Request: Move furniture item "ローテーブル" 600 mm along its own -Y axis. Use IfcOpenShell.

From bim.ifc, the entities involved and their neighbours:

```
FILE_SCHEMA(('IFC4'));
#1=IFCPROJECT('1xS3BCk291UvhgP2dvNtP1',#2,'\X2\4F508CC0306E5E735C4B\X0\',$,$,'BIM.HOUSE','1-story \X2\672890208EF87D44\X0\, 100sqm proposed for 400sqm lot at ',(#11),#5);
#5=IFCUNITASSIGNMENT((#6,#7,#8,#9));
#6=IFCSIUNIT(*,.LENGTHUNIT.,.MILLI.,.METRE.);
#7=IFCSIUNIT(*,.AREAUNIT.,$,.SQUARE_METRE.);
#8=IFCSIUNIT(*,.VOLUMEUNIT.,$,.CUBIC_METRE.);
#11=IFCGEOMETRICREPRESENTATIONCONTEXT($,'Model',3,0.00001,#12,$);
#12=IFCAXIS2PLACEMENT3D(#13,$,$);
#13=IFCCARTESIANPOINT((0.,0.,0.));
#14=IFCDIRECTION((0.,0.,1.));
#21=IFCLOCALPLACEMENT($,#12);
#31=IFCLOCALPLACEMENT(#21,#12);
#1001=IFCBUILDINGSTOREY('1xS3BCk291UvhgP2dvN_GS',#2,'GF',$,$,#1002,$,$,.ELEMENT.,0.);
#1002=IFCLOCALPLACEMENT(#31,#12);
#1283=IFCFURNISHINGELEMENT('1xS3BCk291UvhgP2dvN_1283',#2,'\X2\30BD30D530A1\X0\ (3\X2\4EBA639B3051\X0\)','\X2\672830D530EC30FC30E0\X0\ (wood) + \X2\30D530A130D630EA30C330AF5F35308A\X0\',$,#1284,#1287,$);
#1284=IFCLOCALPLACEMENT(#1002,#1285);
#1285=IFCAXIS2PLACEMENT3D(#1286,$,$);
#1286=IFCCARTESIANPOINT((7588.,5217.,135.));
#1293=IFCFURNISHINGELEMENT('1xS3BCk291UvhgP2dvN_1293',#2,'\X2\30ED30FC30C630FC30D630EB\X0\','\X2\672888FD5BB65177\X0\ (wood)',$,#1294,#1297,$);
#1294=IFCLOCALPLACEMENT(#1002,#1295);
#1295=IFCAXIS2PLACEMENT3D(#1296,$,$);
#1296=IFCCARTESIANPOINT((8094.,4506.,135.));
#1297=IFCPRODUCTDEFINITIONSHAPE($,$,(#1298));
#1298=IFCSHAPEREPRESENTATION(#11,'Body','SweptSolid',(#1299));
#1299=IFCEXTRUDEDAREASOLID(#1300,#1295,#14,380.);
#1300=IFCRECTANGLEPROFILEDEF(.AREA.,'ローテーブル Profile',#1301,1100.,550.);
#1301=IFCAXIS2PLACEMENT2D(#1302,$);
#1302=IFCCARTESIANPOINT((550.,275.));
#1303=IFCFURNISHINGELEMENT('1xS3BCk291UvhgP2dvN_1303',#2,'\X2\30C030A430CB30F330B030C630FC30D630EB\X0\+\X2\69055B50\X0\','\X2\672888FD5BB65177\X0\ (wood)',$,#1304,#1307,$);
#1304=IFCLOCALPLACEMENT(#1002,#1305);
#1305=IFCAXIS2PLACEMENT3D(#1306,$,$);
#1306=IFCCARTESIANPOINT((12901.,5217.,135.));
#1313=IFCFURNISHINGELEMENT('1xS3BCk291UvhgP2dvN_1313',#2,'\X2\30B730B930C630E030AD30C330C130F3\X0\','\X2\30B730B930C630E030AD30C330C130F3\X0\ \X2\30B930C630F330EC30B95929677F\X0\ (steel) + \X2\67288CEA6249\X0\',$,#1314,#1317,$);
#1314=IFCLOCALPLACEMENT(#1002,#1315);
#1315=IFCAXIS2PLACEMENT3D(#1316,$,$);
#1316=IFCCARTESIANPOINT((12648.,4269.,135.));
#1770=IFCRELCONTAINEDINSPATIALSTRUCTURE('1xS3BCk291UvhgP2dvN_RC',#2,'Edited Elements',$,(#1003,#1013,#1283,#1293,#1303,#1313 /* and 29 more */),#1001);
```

```python
import ifcopenshell
import ifcopenshell.api.geometry
import ifcopenshell.util.placement

model = ifcopenshell.open("bim.ifc")

item = model.by_guid("1xS3BCk291UvhgP2dvN_1293")
matrix = ifcopenshell.util.placement.get_local_placement(item.ObjectPlacement)
matrix[:3, 3] -= matrix[:3, 1] * 600.0
ifcopenshell.api.geometry.edit_object_placement(model, product=item, matrix=matrix, is_si=False)

print(ifcopenshell.util.placement.get_local_placement(item.ObjectPlacement).round(3) + 0.0)

model.write("bim_v2.ifc")
```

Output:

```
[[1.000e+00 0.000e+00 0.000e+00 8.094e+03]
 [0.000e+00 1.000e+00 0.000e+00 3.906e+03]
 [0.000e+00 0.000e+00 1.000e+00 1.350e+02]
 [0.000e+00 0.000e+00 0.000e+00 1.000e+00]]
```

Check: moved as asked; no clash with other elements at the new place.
